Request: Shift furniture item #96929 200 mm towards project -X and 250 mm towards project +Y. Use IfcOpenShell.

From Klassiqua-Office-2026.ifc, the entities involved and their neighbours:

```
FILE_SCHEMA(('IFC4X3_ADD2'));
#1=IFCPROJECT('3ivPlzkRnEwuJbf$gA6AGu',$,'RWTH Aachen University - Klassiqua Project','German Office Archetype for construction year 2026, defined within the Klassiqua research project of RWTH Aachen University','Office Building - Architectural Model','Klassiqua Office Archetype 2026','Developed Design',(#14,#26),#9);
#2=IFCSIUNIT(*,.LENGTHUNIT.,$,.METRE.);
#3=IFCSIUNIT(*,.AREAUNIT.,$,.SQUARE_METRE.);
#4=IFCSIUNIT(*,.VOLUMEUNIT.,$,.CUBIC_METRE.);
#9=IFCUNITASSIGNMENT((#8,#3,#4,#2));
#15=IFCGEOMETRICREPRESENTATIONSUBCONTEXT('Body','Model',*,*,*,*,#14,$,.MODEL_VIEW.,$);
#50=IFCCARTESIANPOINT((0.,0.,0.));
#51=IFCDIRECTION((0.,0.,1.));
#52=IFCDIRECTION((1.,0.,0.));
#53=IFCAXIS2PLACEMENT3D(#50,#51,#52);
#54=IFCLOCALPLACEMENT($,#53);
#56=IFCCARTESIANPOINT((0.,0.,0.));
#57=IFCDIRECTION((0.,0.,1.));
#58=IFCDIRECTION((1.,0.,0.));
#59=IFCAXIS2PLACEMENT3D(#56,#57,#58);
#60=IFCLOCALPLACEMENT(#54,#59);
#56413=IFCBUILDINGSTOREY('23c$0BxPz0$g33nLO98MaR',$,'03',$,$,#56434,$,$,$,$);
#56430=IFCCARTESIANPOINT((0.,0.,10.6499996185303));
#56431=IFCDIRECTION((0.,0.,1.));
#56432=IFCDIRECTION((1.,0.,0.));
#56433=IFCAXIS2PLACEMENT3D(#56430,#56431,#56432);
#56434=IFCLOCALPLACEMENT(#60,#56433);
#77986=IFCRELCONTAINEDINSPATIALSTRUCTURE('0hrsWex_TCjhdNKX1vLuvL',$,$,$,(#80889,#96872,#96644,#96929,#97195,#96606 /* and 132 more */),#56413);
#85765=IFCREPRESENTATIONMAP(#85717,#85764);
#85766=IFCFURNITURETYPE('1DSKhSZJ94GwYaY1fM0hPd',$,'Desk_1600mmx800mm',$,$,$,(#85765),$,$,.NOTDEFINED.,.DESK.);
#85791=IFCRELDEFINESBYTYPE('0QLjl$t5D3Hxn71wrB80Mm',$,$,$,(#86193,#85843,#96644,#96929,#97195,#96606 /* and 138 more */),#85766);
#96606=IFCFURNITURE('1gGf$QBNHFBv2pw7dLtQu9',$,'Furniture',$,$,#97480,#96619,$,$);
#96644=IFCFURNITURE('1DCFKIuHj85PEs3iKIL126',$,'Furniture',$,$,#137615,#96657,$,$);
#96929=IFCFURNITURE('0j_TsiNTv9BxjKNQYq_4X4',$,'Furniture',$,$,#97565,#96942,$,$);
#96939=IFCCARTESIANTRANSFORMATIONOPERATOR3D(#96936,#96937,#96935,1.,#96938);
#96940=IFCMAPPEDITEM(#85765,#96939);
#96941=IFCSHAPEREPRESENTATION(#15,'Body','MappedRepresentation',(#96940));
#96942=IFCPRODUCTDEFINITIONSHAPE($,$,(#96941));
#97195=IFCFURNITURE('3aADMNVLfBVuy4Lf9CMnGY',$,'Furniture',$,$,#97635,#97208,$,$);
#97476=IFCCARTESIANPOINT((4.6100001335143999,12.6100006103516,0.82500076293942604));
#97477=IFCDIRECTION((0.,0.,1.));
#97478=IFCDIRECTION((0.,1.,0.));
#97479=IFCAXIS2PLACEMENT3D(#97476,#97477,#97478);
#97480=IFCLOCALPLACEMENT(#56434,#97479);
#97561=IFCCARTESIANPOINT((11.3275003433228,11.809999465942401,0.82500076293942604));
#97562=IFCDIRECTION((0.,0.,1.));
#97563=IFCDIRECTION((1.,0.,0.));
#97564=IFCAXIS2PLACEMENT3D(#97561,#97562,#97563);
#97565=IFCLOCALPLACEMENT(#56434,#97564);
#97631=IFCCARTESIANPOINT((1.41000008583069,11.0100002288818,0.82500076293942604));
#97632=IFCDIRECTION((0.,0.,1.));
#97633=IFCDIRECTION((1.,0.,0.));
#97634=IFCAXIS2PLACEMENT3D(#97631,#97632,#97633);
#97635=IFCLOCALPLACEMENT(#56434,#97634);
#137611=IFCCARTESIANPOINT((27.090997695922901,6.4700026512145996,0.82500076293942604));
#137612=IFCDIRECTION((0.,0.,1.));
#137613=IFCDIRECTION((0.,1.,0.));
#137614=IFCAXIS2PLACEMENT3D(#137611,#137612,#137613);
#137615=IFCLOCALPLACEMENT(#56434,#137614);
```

```python
import ifcopenshell
import ifcopenshell.api.geometry
import ifcopenshell.util.placement
import ifcopenshell.util.unit

model = ifcopenshell.open("Klassiqua-Office-2026.ifc")
unit_scale = ifcopenshell.util.unit.calculate_unit_scale(model)

item = model.by_guid("0j_TsiNTv9BxjKNQYq_4X4")
matrix = ifcopenshell.util.placement.get_local_placement(item.ObjectPlacement)
matrix[0, 3] -= 0.2 / unit_scale
matrix[1, 3] += 0.25 / unit_scale
ifcopenshell.api.geometry.edit_object_placement(model, product=item, matrix=matrix, is_si=False)

print(ifcopenshell.util.placement.get_local_placement(item.ObjectPlacement).round(3) + 0.0)

model.write("Klassiqua-Office-2026_edited.ifc")
```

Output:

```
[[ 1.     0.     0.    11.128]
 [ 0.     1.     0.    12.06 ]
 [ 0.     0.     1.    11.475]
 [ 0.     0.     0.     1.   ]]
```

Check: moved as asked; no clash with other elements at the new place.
